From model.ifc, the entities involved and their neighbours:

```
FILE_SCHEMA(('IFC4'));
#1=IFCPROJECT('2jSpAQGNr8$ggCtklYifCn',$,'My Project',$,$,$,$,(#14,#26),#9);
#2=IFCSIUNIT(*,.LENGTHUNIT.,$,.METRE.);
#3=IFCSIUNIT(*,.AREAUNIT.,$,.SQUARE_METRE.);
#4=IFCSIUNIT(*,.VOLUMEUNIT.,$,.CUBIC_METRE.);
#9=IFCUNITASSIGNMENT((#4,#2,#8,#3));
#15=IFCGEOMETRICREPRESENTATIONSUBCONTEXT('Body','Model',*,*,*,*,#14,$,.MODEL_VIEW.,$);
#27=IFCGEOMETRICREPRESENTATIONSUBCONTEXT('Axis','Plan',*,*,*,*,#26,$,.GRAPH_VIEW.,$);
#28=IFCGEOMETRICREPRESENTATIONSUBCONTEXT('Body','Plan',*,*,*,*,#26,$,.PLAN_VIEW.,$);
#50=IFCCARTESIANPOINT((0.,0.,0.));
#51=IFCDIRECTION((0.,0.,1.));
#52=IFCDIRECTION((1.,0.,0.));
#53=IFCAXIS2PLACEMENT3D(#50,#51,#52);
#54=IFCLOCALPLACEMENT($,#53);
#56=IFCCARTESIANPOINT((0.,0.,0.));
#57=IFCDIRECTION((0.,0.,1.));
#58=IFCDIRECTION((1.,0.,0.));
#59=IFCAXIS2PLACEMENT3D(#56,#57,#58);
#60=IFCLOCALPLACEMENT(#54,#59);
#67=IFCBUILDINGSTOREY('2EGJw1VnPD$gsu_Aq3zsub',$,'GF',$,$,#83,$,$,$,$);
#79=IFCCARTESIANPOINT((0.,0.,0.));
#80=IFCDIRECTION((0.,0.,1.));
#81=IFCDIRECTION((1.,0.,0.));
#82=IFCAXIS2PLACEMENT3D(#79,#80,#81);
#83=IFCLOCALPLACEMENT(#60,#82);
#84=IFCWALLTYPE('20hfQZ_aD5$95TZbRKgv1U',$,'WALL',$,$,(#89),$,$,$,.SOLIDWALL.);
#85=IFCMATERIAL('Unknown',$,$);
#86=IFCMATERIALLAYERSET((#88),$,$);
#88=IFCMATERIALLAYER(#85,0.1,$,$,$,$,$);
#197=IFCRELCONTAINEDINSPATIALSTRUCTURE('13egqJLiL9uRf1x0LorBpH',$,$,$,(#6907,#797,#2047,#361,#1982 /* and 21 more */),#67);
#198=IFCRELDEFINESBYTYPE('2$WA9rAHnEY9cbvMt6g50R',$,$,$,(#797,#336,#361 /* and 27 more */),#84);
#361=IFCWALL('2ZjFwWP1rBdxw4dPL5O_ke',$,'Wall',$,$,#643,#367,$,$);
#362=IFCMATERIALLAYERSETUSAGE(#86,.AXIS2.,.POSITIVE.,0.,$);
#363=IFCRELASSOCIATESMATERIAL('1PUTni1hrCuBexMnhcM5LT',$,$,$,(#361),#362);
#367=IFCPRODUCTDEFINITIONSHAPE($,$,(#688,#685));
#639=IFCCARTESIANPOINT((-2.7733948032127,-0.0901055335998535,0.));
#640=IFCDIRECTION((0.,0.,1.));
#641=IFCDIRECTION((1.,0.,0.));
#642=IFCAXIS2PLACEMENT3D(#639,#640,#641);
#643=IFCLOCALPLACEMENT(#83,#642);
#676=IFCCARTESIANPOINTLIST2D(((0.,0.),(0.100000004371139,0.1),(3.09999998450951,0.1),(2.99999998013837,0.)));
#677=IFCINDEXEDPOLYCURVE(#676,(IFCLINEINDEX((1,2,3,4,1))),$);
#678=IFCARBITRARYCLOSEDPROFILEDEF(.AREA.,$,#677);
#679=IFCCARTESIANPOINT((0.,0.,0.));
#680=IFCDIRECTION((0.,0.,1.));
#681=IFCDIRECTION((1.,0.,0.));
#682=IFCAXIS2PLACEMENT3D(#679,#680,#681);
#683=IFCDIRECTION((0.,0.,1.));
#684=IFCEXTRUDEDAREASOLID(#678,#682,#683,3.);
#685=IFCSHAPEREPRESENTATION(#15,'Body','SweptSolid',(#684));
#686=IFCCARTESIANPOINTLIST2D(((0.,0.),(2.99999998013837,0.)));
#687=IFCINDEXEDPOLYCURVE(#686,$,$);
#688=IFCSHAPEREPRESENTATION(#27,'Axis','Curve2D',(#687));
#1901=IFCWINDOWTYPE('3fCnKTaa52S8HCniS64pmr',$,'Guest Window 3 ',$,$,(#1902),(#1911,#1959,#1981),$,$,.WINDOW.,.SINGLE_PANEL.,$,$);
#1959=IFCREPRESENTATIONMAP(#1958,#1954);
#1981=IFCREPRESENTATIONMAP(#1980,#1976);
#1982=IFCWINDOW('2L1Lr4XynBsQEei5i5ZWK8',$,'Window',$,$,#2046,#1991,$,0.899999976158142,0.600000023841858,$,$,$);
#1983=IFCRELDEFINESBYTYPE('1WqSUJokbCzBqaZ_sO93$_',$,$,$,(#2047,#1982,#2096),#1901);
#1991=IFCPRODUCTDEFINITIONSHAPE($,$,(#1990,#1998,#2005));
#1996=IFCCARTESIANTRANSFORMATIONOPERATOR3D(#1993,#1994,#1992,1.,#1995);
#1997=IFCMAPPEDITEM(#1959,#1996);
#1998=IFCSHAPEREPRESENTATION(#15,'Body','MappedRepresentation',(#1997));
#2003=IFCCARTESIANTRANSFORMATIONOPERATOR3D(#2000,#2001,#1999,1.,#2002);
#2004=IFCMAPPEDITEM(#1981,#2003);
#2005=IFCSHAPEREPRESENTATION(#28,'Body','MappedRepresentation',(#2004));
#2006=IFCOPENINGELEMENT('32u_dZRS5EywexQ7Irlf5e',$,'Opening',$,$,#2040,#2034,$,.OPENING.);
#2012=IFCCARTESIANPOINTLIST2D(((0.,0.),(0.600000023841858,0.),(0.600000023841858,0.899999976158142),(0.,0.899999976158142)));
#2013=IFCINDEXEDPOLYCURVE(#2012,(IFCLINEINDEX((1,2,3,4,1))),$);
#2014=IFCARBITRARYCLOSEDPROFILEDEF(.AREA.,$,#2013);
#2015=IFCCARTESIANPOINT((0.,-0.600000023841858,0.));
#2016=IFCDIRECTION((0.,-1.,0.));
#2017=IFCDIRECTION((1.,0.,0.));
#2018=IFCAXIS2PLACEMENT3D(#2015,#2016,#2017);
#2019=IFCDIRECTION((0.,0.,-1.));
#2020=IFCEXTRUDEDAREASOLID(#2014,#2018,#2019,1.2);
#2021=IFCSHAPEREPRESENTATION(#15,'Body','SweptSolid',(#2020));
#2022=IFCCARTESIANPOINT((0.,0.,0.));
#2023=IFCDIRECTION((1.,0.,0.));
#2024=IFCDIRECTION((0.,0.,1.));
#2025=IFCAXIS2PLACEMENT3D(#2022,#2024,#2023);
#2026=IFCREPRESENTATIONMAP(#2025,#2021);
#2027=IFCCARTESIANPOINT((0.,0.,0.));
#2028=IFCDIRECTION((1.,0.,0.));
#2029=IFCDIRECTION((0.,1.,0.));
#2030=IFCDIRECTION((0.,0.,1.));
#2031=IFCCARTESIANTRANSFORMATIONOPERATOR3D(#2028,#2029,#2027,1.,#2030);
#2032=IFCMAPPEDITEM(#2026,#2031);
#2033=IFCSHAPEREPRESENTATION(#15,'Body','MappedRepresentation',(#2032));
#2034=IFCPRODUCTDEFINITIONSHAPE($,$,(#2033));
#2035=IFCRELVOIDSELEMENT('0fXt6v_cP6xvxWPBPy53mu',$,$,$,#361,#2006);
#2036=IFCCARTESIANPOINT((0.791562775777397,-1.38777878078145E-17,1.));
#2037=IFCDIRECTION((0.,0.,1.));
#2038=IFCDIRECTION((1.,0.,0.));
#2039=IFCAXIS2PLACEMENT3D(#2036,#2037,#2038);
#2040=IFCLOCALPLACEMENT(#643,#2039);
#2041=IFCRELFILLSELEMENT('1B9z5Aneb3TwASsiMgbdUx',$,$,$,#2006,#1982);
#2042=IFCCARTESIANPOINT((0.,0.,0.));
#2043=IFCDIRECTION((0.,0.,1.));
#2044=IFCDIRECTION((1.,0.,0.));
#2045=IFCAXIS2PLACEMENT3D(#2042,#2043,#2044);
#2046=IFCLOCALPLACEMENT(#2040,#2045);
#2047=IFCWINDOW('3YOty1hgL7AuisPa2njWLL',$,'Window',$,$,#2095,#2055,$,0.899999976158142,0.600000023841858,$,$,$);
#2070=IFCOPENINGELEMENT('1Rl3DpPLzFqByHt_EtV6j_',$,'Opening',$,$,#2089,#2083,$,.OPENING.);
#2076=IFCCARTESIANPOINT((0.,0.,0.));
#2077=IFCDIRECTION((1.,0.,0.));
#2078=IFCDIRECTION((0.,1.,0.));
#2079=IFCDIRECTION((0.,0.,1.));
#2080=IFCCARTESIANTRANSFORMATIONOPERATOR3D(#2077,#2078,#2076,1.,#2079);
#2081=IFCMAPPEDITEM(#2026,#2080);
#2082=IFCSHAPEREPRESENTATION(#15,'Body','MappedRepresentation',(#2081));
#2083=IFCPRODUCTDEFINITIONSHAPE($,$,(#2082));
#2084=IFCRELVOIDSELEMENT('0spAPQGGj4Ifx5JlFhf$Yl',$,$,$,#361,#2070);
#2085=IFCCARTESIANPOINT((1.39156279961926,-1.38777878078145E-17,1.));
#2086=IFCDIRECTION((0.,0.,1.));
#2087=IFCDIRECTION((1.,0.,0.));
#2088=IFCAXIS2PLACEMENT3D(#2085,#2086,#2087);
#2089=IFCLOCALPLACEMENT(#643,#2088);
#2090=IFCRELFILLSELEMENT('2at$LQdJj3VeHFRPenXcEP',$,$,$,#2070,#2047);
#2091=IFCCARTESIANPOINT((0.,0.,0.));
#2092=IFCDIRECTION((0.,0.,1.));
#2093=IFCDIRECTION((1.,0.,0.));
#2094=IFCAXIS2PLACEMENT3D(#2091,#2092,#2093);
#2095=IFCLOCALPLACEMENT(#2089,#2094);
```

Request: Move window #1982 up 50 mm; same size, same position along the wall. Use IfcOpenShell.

```python
import numpy as np
import ifcopenshell
import ifcopenshell.api.geometry
import ifcopenshell.util.placement
import ifcopenshell.util.unit

model = ifcopenshell.open("model.ifc")
unit_scale = ifcopenshell.util.unit.calculate_unit_scale(model)

window = model.by_id(1982)
opening = window.FillsVoids[0].RelatingOpeningElement
dz = 0.05

shift = np.array([0.0, 0.0, dz])
# The window is placed relative to its opening, so it follows when the opening moves.
matrix = ifcopenshell.util.placement.get_local_placement(opening.ObjectPlacement)
matrix[:3, 3] += shift
ifcopenshell.api.geometry.edit_object_placement(
    model, product=opening, matrix=matrix, is_si=False, should_transform_children=True
)

print(f"moved by {dz * unit_scale:+.3f} m")

model.write("model_edited.ifc")
```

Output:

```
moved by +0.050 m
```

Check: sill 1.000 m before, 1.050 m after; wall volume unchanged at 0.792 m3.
